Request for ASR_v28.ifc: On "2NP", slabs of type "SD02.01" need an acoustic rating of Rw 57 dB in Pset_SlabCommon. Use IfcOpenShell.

First a look at what the model holds.

```python
import ifcopenshell
import ifcopenshell.util.element

model = ifcopenshell.open("ASR_v28.ifc")
print(model.schema)
storey = next(s for s in model.by_type("IfcBuildingStorey") if s.Name == "2NP")
slabs = [e for e in ifcopenshell.util.element.get_decomposition(storey) if e.is_a("IfcSlab")]
seen = {}
for e in slabs:
    element_type = ifcopenshell.util.element.get_type(e)
    key = (element_type.Name if element_type != e and element_type else None, ifcopenshell.util.element.get_pset(e, "Pset_SlabCommon", "AcousticRating"))
    seen[key] = seen.get(key, 0) + 1
for (name, value), count in sorted(seen.items(), key=str):
    print(count, "x", name, "|", value)
```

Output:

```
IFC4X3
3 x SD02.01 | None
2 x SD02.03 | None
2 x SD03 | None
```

```python
import ifcopenshell
import ifcopenshell.api.pset
import ifcopenshell.util.element

model = ifcopenshell.open("ASR_v28.ifc")

storey = next(s for s in model.by_type("IfcBuildingStorey") if s.Name == "2NP")
slabs = [e for e in ifcopenshell.util.element.get_decomposition(storey) if e.is_a("IfcSlab")]

count = 0
for e in slabs:
    element_type = ifcopenshell.util.element.get_type(e)
    if element_type in (None, e) or element_type.Name != "SD02.01":
        continue
    # add_pset returns the element's existing set when there is one.
    pset = ifcopenshell.api.pset.add_pset(model, product=e, name="Pset_SlabCommon")
    ifcopenshell.api.pset.edit_pset(model, pset=pset, properties={"AcousticRating": "Rw 57 dB"})
    count += 1

print(count, "slabs updated")

model.write("ASR_v28_rev.ifc")
```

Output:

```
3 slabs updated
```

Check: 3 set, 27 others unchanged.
